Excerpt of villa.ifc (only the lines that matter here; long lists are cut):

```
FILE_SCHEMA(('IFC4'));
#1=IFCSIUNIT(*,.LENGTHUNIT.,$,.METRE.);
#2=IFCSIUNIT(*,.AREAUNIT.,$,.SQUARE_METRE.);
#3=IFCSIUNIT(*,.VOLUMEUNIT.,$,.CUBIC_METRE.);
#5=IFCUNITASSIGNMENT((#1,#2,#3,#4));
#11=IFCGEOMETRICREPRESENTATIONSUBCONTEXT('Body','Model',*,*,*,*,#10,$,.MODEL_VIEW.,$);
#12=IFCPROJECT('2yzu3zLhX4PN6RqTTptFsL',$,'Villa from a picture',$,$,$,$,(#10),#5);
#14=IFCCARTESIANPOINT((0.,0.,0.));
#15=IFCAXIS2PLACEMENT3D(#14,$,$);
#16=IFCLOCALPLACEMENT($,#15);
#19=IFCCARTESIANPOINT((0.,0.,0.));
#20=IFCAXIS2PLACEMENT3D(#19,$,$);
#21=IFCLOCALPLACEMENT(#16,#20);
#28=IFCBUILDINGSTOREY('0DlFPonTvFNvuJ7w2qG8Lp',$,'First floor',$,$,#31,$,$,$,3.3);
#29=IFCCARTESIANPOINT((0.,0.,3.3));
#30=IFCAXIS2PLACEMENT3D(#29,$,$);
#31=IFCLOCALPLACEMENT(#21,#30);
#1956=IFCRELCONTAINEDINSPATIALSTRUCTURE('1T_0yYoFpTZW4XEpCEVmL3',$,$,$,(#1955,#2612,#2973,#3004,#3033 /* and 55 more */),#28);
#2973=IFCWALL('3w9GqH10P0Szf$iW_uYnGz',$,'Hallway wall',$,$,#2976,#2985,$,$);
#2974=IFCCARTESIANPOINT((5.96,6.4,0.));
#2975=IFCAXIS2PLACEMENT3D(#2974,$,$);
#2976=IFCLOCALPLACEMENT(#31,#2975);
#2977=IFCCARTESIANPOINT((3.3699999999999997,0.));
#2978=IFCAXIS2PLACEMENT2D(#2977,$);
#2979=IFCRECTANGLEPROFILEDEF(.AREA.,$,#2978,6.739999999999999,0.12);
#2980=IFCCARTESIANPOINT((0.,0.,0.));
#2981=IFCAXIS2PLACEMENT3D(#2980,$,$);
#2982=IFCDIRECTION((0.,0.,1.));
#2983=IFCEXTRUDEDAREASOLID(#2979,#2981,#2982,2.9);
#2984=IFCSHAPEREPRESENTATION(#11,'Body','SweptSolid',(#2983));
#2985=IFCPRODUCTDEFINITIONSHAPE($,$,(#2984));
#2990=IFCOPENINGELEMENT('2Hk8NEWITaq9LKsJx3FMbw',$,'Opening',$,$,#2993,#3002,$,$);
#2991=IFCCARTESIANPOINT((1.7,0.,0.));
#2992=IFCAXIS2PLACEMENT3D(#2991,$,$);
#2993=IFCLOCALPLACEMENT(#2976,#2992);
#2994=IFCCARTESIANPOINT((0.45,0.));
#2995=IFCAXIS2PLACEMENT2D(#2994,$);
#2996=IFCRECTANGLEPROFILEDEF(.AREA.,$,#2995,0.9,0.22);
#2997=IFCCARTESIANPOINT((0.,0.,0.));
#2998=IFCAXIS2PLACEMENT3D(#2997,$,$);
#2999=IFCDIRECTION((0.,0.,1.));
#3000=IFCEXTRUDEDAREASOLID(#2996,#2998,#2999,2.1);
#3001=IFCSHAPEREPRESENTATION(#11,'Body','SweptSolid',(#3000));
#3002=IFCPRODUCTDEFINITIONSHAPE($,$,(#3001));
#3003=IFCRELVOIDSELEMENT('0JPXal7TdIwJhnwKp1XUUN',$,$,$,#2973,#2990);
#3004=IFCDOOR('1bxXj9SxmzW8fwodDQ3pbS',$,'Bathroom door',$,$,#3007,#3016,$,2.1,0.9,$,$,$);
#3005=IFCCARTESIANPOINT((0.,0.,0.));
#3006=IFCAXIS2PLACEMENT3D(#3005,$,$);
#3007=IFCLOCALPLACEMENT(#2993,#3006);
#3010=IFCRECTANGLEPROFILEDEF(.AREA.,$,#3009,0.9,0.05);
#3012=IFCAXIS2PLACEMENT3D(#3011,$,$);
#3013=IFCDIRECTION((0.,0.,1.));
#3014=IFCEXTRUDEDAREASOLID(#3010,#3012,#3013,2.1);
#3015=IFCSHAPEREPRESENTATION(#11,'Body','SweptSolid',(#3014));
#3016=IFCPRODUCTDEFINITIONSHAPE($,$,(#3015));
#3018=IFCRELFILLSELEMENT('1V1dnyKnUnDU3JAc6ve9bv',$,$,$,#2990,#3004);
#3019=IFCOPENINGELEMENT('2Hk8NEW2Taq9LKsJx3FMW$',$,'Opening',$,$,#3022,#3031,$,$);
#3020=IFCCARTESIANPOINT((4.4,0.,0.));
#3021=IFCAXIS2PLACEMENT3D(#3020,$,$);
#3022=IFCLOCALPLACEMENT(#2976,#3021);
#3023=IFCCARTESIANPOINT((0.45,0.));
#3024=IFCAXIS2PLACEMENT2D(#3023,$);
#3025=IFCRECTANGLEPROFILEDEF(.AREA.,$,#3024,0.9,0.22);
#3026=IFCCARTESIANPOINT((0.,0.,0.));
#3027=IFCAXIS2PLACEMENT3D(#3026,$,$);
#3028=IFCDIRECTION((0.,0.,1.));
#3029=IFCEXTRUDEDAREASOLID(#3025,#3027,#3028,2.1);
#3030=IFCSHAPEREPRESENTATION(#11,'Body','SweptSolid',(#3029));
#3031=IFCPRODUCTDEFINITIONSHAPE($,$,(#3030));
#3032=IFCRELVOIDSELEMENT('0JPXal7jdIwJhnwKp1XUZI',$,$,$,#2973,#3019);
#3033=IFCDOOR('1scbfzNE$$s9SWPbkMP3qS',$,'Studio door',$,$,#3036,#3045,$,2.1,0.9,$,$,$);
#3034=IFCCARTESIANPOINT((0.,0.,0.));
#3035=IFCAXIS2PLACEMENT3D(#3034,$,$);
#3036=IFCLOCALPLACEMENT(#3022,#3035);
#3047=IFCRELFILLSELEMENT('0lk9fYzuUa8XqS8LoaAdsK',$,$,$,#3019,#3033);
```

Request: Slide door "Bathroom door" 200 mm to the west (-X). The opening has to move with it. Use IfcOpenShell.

```python
import ifcopenshell
import ifcopenshell.api.geometry
import ifcopenshell.util.placement
import ifcopenshell.util.unit

model = ifcopenshell.open("villa.ifc")
unit_scale = ifcopenshell.util.unit.calculate_unit_scale(model)

door = model.by_guid("1bxXj9SxmzW8fwodDQ3pbS")
opening = door.FillsVoids[0].RelatingOpeningElement
wall = opening.VoidsElements[0].RelatingBuildingElement

wall_matrix = ifcopenshell.util.placement.get_local_placement(wall.ObjectPlacement)
shift = wall_matrix[:3, 0] * -0.2 / unit_scale
before = ifcopenshell.util.placement.get_local_placement(door.ObjectPlacement)[:3, 3].copy()

# The door is placed relative to its opening, so it follows when the opening moves.
matrix = ifcopenshell.util.placement.get_local_placement(opening.ObjectPlacement)
matrix[:3, 3] += shift
ifcopenshell.api.geometry.edit_object_placement(
    model, product=opening, matrix=matrix, is_si=False, should_transform_children=True
)

after = ifcopenshell.util.placement.get_local_placement(door.ObjectPlacement)[:3, 3]
print("door moved by", (after - before).round(3) + 0.0)

model.write("villa_edited.ifc")
```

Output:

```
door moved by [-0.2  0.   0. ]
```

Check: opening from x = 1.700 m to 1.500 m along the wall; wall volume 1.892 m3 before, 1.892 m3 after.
